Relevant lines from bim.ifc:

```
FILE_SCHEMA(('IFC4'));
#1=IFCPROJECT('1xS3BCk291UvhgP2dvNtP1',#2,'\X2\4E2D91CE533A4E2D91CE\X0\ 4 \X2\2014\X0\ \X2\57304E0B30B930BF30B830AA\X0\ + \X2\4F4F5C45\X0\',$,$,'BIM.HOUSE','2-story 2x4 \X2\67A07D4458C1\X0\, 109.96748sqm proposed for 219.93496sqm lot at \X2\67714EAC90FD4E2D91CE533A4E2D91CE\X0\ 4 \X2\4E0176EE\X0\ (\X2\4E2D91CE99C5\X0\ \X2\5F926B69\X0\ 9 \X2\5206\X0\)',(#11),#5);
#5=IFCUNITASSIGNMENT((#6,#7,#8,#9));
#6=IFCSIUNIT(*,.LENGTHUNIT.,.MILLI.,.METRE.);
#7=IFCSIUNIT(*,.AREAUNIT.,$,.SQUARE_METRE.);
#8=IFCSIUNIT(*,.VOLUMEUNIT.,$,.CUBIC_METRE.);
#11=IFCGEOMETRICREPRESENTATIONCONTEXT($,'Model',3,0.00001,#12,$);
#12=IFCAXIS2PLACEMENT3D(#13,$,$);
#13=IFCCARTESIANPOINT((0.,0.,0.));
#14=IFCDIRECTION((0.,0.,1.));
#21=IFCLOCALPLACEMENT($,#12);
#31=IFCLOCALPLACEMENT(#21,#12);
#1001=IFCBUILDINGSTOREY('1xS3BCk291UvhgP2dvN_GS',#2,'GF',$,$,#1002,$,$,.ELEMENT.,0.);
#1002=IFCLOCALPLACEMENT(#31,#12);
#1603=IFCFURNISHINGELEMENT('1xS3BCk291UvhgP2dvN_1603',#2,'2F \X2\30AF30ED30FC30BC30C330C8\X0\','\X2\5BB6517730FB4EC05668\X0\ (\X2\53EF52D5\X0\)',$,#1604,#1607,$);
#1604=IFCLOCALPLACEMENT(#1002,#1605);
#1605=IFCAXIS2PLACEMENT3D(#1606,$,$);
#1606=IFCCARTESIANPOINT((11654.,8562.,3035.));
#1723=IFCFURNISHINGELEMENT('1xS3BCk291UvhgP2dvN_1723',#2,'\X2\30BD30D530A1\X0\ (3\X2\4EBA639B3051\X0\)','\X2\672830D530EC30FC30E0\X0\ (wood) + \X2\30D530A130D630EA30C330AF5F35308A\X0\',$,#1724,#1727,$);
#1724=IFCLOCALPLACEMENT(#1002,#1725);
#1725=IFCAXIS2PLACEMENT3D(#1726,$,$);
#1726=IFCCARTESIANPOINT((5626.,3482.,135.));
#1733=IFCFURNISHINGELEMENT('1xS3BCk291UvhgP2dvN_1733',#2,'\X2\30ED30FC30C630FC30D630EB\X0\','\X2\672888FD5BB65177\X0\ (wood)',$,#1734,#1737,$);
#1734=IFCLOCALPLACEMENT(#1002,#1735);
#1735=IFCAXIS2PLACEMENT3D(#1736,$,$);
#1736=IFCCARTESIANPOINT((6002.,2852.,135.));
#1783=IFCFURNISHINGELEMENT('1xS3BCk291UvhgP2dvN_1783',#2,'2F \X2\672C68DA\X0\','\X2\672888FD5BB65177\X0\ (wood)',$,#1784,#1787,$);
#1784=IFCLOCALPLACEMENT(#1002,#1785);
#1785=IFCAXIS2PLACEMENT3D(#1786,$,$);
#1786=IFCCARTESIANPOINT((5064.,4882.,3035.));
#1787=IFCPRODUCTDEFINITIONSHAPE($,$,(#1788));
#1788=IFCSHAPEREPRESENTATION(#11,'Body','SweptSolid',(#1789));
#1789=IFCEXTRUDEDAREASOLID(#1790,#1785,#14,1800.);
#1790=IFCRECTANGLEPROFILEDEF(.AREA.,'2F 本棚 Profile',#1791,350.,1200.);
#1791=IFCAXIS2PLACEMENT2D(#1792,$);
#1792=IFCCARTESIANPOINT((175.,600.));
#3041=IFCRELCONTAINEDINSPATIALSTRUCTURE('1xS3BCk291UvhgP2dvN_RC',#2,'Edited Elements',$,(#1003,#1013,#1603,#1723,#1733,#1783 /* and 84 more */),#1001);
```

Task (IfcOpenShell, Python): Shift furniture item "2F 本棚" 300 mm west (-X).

```python
import ifcopenshell
import ifcopenshell.api.geometry
import ifcopenshell.util.placement

model = ifcopenshell.open("bim.ifc")

item = model.by_guid("1xS3BCk291UvhgP2dvN_1783")
matrix = ifcopenshell.util.placement.get_local_placement(item.ObjectPlacement)
matrix[0, 3] -= 300.0
ifcopenshell.api.geometry.edit_object_placement(model, product=item, matrix=matrix, is_si=False)

print(ifcopenshell.util.placement.get_local_placement(item.ObjectPlacement).round(3) + 0.0)

model.write("bim_edited.ifc")
```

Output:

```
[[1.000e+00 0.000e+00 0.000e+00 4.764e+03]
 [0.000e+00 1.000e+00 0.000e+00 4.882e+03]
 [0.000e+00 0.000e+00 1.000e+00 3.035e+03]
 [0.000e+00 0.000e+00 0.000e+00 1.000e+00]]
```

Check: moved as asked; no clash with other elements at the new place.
